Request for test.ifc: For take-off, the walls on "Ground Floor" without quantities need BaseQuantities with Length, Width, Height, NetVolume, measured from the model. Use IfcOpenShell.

First a look at what the model holds.

```python
import ifcopenshell
import ifcopenshell.util.element
import ifcopenshell.util.unit

model = ifcopenshell.open("test.ifc")
print(model.schema)
for unit_type in ("LENGTHUNIT", "AREAUNIT", "VOLUMEUNIT"):
    print(unit_type, ifcopenshell.util.unit.calculate_unit_scale(model, unit_type))
storey = next(s for s in model.by_type("IfcBuildingStorey") if s.Name == "Ground Floor")
walls = [e for e in ifcopenshell.util.element.get_decomposition(storey) if e.is_a("IfcWall")]
for e in sorted(walls, key=lambda e: e.id()):
    print(e.id(), e.is_a(), e.Name, list(ifcopenshell.util.element.get_psets(e, qtos_only=True)), sep=" | ")
```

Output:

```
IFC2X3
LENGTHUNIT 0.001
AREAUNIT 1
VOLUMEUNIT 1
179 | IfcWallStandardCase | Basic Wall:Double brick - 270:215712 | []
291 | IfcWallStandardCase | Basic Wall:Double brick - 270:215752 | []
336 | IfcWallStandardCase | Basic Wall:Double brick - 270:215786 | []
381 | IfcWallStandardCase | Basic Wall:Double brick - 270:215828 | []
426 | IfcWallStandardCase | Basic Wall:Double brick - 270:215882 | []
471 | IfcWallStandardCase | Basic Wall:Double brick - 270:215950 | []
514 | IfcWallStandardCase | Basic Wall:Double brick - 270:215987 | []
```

```python
import ifcopenshell
import ifcopenshell.api.pset
import ifcopenshell.geom
import ifcopenshell.util.element
import ifcopenshell.util.shape
import ifcopenshell.util.unit

model = ifcopenshell.open("test.ifc")
unit_scale = ifcopenshell.util.unit.calculate_unit_scale(model)
volume_scale = ifcopenshell.util.unit.calculate_unit_scale(model, "VOLUMEUNIT")
settings = ifcopenshell.geom.settings()

storey = next(s for s in model.by_type("IfcBuildingStorey") if s.Name == "Ground Floor")
walls = [e for e in ifcopenshell.util.element.get_decomposition(storey) if e.is_a("IfcWall")]

for e in sorted(walls, key=lambda e: e.id()):
    if ifcopenshell.util.element.get_psets(e, qtos_only=True, should_inherit=False):
        continue
    # Geometry comes back in metres, in the element's own axes.
    shape = ifcopenshell.geom.create_shape(settings, e)
    values = {
        "Length": ifcopenshell.util.shape.get_x(shape.geometry) / unit_scale,
        "Width": ifcopenshell.util.shape.get_y(shape.geometry) / unit_scale,
        "Height": ifcopenshell.util.shape.get_z(shape.geometry) / unit_scale,
        "NetVolume": ifcopenshell.util.shape.get_volume(shape.geometry) / volume_scale,
    }
    qto = ifcopenshell.api.pset.add_qto(model, product=e, name="BaseQuantities")
    ifcopenshell.api.pset.edit_qto(model, qto=qto, properties=values)
    print(e.id(), {k: round(v, 3) for k, v in values.items()})

model.write("test_rev.ifc")
```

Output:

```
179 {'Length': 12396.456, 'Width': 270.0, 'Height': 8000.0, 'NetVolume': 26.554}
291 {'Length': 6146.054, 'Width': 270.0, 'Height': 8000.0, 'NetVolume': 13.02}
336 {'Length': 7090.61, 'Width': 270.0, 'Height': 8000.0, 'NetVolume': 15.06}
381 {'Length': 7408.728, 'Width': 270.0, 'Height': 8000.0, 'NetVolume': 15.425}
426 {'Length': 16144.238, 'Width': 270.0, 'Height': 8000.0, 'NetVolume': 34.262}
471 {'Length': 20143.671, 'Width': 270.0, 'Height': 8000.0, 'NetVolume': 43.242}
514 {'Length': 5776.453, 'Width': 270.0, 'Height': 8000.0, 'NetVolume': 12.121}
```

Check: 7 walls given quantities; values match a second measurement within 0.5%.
